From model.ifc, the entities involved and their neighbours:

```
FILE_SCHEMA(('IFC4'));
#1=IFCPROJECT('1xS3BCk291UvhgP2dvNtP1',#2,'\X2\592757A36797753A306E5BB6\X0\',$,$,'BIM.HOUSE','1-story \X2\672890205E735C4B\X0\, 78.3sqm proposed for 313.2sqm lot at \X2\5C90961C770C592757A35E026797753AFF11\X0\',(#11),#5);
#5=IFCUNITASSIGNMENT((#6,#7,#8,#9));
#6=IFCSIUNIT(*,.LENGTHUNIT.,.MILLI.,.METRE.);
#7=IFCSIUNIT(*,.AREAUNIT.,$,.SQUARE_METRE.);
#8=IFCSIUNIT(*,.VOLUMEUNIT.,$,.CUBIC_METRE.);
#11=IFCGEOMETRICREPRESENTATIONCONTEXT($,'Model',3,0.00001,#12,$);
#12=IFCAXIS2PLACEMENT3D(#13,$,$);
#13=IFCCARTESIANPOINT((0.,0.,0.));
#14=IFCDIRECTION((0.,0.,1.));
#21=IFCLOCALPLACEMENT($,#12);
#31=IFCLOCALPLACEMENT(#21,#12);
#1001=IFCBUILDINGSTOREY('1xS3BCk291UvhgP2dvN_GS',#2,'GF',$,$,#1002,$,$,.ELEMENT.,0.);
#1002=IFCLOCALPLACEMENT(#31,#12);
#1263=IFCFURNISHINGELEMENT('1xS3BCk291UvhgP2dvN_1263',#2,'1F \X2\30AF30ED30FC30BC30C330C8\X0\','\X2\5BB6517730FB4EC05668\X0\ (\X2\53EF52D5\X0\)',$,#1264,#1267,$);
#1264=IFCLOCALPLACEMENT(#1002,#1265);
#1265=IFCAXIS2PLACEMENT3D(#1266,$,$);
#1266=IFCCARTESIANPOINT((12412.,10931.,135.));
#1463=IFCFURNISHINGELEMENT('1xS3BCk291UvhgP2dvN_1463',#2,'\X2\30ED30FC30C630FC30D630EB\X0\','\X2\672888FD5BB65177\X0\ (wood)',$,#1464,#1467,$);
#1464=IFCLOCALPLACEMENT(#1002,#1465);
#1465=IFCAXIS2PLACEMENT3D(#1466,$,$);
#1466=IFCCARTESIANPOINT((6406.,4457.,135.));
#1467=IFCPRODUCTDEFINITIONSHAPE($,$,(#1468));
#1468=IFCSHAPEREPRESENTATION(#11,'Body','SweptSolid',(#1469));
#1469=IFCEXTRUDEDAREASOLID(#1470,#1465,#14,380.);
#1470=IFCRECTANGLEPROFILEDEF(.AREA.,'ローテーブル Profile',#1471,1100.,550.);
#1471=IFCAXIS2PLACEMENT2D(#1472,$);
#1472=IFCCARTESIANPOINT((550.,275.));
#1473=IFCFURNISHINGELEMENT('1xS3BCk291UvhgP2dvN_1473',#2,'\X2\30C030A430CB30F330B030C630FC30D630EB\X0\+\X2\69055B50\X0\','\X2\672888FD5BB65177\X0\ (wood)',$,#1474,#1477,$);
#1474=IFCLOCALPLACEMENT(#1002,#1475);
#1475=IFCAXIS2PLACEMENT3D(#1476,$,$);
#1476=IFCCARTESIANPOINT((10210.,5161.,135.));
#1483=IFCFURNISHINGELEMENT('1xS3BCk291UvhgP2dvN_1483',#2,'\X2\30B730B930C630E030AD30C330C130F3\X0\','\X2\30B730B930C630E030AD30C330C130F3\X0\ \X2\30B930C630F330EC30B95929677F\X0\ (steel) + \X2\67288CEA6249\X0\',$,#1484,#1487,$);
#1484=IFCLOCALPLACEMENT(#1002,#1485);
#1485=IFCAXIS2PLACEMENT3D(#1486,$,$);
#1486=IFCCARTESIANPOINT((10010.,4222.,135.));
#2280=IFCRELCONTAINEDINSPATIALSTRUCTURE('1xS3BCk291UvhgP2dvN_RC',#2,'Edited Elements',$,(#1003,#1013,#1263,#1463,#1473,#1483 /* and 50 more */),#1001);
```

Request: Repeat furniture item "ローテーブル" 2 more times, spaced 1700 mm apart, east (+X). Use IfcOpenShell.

```python
import numpy as np
import ifcopenshell
import ifcopenshell.api.geometry
import ifcopenshell.api.root
import ifcopenshell.util.element
import ifcopenshell.util.placement

model = ifcopenshell.open("model.ifc")


def reuse_history(source, copy):
    """copy_class also copies each property set's owner history, people and application; keep the originals."""
    for rel in copy.IsDefinedBy:
        if rel.is_a("IfcRelDefinesByProperties") and (history := rel.RelatingPropertyDefinition.OwnerHistory):
            rel.RelatingPropertyDefinition.OwnerHistory = source.OwnerHistory
            ifcopenshell.util.element.remove_deep2(model, history)


source = model.by_id(1463)
base = ifcopenshell.util.placement.get_local_placement(source.ObjectPlacement)
step = np.array([1.0, 0.0, 0.0]) * 1700.0

for i in range(1, 3):
    copy = ifcopenshell.api.root.copy_class(model, product=source)
    copy.Representation = ifcopenshell.util.element.copy_deep(
        model, source.Representation, exclude=["IfcGeometricRepresentationContext", "IfcRepresentationMap"]
    )
    reuse_history(source, copy)
    matrix = base.copy()
    matrix[:3, 3] += i * step
    print("added at", matrix[:3, 3].round(3) + 0.0)
    ifcopenshell.api.geometry.edit_object_placement(model, product=copy, matrix=matrix, is_si=False)

model.write("model-out.ifc")
```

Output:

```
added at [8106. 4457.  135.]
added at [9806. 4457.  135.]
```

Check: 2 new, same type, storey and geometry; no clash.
